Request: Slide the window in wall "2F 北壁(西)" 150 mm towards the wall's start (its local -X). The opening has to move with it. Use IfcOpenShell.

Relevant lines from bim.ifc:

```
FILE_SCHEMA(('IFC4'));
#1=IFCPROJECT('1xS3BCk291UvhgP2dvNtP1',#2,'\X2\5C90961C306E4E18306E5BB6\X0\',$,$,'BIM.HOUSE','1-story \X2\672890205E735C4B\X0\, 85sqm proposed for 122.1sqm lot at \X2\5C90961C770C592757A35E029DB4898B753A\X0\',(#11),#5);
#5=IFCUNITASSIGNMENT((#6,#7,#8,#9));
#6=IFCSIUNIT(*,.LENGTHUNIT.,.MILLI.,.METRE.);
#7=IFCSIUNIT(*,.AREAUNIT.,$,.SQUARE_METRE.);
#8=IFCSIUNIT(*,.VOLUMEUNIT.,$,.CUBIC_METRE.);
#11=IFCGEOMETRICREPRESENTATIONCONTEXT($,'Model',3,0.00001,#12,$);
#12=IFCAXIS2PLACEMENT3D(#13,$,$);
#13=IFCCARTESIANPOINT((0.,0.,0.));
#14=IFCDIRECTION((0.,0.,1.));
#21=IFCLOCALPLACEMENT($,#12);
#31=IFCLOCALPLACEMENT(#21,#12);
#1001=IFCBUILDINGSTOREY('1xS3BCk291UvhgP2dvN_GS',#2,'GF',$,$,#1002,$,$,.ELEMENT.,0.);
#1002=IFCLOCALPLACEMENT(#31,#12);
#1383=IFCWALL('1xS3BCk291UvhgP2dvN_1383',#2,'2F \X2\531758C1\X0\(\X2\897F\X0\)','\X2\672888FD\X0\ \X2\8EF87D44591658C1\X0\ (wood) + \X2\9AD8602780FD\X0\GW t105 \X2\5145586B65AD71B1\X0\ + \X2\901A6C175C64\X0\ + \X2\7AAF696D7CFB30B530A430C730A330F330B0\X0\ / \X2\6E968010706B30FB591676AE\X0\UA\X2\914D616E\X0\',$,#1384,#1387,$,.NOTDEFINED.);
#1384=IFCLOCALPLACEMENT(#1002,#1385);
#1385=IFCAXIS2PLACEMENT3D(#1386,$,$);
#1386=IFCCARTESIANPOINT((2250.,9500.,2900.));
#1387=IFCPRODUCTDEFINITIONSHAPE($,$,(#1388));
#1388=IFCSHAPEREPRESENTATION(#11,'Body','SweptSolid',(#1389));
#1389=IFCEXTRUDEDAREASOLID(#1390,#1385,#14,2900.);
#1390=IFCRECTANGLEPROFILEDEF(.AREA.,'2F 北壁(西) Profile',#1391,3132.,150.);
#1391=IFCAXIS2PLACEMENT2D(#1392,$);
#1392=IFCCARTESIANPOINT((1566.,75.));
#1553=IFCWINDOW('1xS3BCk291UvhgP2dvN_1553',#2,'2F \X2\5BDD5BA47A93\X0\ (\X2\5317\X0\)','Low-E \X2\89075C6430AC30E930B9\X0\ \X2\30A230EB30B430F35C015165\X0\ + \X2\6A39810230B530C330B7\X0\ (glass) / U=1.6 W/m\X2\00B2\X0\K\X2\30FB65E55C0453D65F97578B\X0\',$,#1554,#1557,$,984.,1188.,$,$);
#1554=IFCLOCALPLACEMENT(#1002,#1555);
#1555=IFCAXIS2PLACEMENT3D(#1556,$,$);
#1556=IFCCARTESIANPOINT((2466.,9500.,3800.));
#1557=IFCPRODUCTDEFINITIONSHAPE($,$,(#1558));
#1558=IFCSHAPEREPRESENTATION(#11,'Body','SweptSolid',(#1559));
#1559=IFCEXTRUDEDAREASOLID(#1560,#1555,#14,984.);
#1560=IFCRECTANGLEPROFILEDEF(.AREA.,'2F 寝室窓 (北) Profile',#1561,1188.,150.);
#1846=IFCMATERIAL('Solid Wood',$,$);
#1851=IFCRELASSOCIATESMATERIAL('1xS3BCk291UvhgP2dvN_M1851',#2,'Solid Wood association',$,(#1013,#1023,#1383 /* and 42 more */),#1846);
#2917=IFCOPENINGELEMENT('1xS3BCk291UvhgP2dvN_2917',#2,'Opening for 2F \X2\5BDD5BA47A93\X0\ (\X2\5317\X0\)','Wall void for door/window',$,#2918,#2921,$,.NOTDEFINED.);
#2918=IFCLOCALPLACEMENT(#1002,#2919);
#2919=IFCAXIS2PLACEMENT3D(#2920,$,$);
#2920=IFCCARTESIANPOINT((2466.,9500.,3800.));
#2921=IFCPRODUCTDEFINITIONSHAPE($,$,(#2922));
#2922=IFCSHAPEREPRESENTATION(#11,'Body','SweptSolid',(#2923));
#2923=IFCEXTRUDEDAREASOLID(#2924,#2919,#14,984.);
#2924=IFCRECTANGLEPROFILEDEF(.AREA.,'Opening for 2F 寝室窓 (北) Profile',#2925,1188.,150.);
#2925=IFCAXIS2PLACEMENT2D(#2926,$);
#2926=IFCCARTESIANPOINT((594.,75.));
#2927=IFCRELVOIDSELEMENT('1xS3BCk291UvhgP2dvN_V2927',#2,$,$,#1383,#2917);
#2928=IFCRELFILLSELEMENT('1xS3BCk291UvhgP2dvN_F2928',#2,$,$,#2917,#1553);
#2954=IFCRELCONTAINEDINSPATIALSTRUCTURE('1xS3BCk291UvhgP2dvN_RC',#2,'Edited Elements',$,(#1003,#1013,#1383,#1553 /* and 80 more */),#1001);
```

```python
import ifcopenshell
import ifcopenshell.api.geometry
import ifcopenshell.util.placement
import ifcopenshell.util.unit

model = ifcopenshell.open("bim.ifc")
unit_scale = ifcopenshell.util.unit.calculate_unit_scale(model)

window = model.by_id(1553)
opening = window.FillsVoids[0].RelatingOpeningElement
wall = opening.VoidsElements[0].RelatingBuildingElement

wall_matrix = ifcopenshell.util.placement.get_local_placement(wall.ObjectPlacement)
shift = wall_matrix[:3, 0] * -0.15 / unit_scale
before = ifcopenshell.util.placement.get_local_placement(window.ObjectPlacement)[:3, 3].copy()

# The window is not placed relative to its opening, so move both.
for product in (opening, window):
    matrix = ifcopenshell.util.placement.get_local_placement(product.ObjectPlacement)
    matrix[:3, 3] += shift
    ifcopenshell.api.geometry.edit_object_placement(model, product=product, matrix=matrix, is_si=False)

after = ifcopenshell.util.placement.get_local_placement(window.ObjectPlacement)[:3, 3]
print("window moved by", (after - before).round(3) + 0.0)

model.write("bim_v2.ifc")
```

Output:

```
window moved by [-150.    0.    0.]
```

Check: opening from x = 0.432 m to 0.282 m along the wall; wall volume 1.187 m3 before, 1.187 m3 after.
